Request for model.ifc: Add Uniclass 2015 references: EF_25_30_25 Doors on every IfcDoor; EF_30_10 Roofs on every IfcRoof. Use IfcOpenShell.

First a look at what the model holds.

```python
import ifcopenshell

model = ifcopenshell.open("model.ifc")
print(model.schema)
print("classifications:", [c.Name for c in model.by_type("IfcClassification")])
for ifc_class in ("IfcDoor", "IfcRoof", "IfcStair", "IfcWall", "IfcWindow"):
    print(ifc_class, len(model.by_type(ifc_class)))
```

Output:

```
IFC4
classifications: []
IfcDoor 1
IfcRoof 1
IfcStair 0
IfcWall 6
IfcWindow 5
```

```python
import ifcopenshell
import ifcopenshell.api.classification

model = ifcopenshell.open("model.ifc")

system = ifcopenshell.api.classification.add_classification(model, classification="Uniclass 2015")

codes = {
    "IfcDoor": ("EF_25_30_25", "Doors"),
    "IfcRoof": ("EF_30_10", "Roofs"),
}
for ifc_class, (code, name) in codes.items():
    products = model.by_type(ifc_class)
    ifcopenshell.api.classification.add_reference(
        model, products=products, classification=system, identification=code, name=name
    )
    print(code, len(products))

model.write("model_updated.ifc")
```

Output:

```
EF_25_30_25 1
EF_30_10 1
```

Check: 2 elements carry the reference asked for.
